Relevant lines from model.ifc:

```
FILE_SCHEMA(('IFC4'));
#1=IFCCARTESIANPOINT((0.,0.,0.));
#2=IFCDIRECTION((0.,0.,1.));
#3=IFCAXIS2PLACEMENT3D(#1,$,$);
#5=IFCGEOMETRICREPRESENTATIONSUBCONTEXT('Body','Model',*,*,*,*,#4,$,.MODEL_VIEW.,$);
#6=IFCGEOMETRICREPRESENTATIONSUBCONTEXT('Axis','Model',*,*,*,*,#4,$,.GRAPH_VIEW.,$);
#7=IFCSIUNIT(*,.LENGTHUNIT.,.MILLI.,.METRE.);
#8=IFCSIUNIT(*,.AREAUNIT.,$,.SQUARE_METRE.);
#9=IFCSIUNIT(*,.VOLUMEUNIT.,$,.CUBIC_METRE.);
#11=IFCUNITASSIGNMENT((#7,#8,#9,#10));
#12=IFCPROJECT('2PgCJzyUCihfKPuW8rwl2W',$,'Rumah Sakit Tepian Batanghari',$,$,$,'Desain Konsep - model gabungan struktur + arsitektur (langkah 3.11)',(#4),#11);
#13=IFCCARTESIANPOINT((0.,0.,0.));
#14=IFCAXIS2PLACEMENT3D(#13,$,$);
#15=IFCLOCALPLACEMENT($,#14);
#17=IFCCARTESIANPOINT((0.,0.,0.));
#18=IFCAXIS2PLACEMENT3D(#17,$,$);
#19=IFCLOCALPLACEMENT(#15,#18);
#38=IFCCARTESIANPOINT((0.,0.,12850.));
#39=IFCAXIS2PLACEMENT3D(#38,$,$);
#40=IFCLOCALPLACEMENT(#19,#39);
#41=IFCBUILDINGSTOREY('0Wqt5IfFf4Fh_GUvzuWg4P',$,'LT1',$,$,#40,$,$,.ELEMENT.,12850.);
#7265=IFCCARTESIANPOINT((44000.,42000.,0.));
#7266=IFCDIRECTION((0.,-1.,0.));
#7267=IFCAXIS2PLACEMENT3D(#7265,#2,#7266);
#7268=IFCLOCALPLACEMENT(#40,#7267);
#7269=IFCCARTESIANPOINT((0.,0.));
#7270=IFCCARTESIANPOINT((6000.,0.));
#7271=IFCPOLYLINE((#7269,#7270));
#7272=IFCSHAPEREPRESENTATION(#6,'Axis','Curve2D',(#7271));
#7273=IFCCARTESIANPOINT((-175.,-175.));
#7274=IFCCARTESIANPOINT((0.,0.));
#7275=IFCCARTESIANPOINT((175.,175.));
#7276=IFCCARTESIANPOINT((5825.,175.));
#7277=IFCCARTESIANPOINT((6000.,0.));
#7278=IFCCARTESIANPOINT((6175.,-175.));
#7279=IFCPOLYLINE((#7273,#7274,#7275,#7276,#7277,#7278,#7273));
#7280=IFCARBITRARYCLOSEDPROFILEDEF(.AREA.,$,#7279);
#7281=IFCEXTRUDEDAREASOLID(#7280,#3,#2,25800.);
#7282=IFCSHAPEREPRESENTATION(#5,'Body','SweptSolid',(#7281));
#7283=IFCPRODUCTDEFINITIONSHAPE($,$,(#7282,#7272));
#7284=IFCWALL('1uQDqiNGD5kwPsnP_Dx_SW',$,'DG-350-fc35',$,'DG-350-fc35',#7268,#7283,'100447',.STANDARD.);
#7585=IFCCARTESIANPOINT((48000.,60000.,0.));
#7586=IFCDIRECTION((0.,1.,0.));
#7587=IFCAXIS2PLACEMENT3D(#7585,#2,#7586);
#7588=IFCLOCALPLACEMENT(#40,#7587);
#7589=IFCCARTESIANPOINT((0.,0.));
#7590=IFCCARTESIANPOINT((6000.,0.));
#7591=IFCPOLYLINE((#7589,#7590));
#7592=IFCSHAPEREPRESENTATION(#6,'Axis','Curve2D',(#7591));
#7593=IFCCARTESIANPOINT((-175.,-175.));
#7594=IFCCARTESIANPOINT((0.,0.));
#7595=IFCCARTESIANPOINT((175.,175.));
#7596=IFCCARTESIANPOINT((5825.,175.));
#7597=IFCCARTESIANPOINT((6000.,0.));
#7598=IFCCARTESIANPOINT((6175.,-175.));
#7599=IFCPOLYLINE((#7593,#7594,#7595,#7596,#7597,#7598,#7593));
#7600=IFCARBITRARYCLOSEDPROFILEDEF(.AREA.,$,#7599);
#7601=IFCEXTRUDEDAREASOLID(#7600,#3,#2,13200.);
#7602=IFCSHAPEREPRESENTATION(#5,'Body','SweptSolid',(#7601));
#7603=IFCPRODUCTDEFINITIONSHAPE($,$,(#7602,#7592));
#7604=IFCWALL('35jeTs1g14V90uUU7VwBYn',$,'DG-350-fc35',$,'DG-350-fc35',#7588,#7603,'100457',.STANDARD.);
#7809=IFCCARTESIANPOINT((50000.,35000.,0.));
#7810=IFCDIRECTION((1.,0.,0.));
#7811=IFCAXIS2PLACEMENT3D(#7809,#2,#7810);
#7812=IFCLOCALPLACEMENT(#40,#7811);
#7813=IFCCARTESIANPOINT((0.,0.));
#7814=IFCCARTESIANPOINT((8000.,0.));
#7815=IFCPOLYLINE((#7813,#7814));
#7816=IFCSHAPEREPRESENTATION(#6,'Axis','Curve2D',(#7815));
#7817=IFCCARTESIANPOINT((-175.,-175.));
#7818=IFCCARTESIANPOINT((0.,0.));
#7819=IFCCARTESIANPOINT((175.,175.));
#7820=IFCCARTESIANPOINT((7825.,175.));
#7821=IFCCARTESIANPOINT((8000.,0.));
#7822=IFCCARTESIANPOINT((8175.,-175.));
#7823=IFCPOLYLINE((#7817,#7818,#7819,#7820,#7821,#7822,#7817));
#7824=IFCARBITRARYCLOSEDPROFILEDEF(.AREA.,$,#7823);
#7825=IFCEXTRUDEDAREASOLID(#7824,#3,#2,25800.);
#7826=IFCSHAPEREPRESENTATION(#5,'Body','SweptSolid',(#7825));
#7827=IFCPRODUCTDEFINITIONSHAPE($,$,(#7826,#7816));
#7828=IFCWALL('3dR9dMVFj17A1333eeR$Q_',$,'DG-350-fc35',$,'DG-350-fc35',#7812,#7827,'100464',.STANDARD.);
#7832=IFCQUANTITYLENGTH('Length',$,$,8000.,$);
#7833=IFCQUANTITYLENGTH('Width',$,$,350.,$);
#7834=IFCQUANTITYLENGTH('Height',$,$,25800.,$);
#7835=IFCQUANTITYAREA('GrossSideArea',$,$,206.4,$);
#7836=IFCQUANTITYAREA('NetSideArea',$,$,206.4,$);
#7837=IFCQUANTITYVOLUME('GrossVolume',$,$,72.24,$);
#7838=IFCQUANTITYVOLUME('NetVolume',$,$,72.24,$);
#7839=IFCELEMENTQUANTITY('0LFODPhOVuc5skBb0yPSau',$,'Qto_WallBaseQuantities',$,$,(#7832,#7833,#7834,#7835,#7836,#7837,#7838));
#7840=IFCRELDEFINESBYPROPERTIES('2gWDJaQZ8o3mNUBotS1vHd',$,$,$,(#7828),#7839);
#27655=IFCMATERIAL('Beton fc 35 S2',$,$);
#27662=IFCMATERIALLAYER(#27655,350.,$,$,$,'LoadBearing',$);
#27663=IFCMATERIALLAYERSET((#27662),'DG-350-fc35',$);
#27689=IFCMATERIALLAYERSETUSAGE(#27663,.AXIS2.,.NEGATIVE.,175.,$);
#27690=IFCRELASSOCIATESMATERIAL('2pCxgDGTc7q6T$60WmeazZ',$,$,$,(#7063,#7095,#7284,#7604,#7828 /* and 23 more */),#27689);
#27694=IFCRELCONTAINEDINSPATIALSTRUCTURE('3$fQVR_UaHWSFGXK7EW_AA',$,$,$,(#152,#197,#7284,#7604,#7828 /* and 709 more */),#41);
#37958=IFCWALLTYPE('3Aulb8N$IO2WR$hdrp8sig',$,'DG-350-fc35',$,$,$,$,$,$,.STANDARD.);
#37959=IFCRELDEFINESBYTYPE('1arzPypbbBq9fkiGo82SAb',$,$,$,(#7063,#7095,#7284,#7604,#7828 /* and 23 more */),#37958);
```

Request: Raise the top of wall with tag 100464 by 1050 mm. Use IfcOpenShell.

```python
import ifcopenshell
import ifcopenshell.api.pset
import ifcopenshell.geom
import ifcopenshell.util.element
import ifcopenshell.util.representation
import ifcopenshell.util.shape
import ifcopenshell.util.unit

model = ifcopenshell.open("model.ifc")
unit_scale = ifcopenshell.util.unit.calculate_unit_scale(model)
area_scale = ifcopenshell.util.unit.calculate_unit_scale(model, "AREAUNIT")
volume_scale = ifcopenshell.util.unit.calculate_unit_scale(model, "VOLUMEUNIT")
settings = ifcopenshell.geom.settings()


def volume(element):
    """Net volume in cubic metres, openings subtracted."""
    shape = ifcopenshell.geom.create_shape(settings, element)
    return ifcopenshell.util.shape.get_volume(shape.geometry)


wall = model.by_guid("3dR9dMVFj17A1333eeR$Q_")
before = volume(wall)

body = ifcopenshell.util.representation.get_representation(wall, "Model", "Body")
solid = body.Items[0]
old_height = solid.Depth
solid.Depth += 1.05 / unit_scale
after = volume(wall)
thickness = 0.35  # wall thickness in metres

# Update the stored height, areas and volumes.
qto = model.by_id(ifcopenshell.util.element.get_pset(wall, "Qto_WallBaseQuantities", should_inherit=False)["id"])
ifcopenshell.api.pset.edit_qto(model, qto=qto, properties={
    "Height": solid.Depth,
    "GrossSideArea": ifcopenshell.util.element.get_pset(wall, "Qto_WallBaseQuantities", "GrossSideArea") * solid.Depth / old_height,
    "NetSideArea": after / thickness / area_scale,
    "GrossVolume": ifcopenshell.util.element.get_pset(wall, "Qto_WallBaseQuantities", "GrossVolume") * solid.Depth / old_height,
    "NetVolume": after / volume_scale,
})

print(f"height {old_height:g} -> {solid.Depth:g}, volume {before:.3f} -> {after:.3f} m3")

model.write("model_rev.ifc")
```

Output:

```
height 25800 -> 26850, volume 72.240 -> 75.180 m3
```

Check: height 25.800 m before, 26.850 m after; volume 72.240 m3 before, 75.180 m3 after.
